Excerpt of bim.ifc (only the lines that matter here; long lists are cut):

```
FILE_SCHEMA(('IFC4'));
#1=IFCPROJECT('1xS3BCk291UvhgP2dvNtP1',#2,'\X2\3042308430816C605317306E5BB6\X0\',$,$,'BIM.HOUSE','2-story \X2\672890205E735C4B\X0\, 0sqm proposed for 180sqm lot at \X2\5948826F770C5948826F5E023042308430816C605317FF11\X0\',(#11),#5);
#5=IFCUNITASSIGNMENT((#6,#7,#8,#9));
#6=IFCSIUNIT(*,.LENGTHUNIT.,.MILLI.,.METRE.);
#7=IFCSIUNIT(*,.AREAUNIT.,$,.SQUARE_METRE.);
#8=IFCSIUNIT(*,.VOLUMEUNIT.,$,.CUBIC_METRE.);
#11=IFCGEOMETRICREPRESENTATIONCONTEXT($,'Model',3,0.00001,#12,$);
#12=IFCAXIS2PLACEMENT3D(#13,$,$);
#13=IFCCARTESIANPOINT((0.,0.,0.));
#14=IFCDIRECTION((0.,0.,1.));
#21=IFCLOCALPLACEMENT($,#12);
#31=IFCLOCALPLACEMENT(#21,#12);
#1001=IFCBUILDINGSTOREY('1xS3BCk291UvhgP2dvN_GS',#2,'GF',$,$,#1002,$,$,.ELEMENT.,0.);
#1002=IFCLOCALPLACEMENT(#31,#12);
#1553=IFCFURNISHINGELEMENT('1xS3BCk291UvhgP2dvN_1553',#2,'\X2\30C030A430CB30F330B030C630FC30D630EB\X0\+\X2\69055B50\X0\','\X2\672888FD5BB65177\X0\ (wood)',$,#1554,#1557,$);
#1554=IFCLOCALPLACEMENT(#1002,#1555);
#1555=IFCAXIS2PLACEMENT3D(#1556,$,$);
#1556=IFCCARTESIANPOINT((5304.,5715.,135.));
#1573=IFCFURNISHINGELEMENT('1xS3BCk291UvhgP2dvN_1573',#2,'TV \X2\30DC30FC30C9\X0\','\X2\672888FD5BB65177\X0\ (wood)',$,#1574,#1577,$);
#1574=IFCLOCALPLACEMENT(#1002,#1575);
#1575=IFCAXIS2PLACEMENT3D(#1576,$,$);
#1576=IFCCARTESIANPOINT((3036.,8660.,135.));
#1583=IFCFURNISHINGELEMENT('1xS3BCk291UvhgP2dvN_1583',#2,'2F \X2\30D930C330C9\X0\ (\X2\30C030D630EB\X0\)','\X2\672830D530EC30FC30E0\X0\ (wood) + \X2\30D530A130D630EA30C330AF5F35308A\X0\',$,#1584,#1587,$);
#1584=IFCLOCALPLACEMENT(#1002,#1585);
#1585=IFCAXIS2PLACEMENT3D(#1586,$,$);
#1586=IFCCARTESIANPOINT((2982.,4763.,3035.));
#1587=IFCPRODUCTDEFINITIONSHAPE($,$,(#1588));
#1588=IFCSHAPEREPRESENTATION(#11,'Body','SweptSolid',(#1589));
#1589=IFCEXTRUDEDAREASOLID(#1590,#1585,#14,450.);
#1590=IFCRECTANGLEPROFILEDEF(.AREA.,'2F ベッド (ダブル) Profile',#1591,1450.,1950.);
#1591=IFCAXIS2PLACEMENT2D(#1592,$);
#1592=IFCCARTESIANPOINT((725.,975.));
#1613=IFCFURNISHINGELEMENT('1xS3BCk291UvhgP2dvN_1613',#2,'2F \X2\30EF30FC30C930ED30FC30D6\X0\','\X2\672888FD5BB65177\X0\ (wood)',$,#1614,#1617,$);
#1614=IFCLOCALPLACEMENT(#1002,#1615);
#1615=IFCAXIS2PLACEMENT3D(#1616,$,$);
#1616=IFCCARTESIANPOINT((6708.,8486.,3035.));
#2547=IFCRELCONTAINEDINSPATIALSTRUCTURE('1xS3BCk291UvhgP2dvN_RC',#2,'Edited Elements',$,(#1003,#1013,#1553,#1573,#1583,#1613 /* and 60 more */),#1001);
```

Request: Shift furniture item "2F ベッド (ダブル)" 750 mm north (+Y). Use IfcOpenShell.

```python
import ifcopenshell
import ifcopenshell.api.geometry
import ifcopenshell.util.placement
import ifcopenshell.util.unit

model = ifcopenshell.open("bim.ifc")
unit_scale = ifcopenshell.util.unit.calculate_unit_scale(model)

item = model.by_guid("1xS3BCk291UvhgP2dvN_1583")
matrix = ifcopenshell.util.placement.get_local_placement(item.ObjectPlacement)
matrix[1, 3] += 0.75 / unit_scale
ifcopenshell.api.geometry.edit_object_placement(model, product=item, matrix=matrix, is_si=False)

print(ifcopenshell.util.placement.get_local_placement(item.ObjectPlacement).round(3) + 0.0)

model.write("bim_rev.ifc")
```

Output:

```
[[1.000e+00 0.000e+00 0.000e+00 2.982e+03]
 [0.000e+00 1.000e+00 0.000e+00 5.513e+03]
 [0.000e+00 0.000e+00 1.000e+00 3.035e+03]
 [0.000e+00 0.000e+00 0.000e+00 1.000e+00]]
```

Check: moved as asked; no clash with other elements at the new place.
